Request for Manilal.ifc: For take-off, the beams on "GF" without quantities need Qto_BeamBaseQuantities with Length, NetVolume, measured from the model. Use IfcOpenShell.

First a look at what the model holds.

```python
import ifcopenshell
import ifcopenshell.util.element
import ifcopenshell.util.unit

model = ifcopenshell.open("Manilal.ifc")
print(model.schema)
for unit_type in ("LENGTHUNIT", "AREAUNIT", "VOLUMEUNIT"):
    print(unit_type, ifcopenshell.util.unit.calculate_unit_scale(model, unit_type))
storey = next(s for s in model.by_type("IfcBuildingStorey") if s.Name == "GF")
beams = [e for e in ifcopenshell.util.element.get_decomposition(storey) if e.is_a("IfcBeam")]
for e in sorted(beams, key=lambda e: e.id()):
    print(e.id(), e.is_a(), e.Name, list(ifcopenshell.util.element.get_psets(e, qtos_only=True)), sep=" | ")
```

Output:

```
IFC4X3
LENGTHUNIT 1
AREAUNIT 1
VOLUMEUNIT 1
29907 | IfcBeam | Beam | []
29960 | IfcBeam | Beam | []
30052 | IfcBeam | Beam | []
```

```python
import ifcopenshell
import ifcopenshell.api.pset
import ifcopenshell.geom
import ifcopenshell.util.element
import ifcopenshell.util.shape
import ifcopenshell.util.unit

model = ifcopenshell.open("Manilal.ifc")
unit_scale = ifcopenshell.util.unit.calculate_unit_scale(model)
volume_scale = ifcopenshell.util.unit.calculate_unit_scale(model, "VOLUMEUNIT")
settings = ifcopenshell.geom.settings()

storey = next(s for s in model.by_type("IfcBuildingStorey") if s.Name == "GF")
beams = [e for e in ifcopenshell.util.element.get_decomposition(storey) if e.is_a("IfcBeam")]

for e in sorted(beams, key=lambda e: e.id()):
    if ifcopenshell.util.element.get_psets(e, qtos_only=True, should_inherit=False):
        continue
    # Geometry comes back in metres, in the element's own axes.
    shape = ifcopenshell.geom.create_shape(settings, e)
    values = {
        "Length": ifcopenshell.util.shape.get_max_xyz(shape.geometry) / unit_scale,
        "NetVolume": ifcopenshell.util.shape.get_volume(shape.geometry) / volume_scale,
    }
    qto = ifcopenshell.api.pset.add_qto(model, product=e, name="Qto_BeamBaseQuantities")
    ifcopenshell.api.pset.edit_qto(model, qto=qto, properties=values)
    print(e.id(), {k: round(v, 3) for k, v in values.items()})

model.write("Manilal_v2.ifc")
```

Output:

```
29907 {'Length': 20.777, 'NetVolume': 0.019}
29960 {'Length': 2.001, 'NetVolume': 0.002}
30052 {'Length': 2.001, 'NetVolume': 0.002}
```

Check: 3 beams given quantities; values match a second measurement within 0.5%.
